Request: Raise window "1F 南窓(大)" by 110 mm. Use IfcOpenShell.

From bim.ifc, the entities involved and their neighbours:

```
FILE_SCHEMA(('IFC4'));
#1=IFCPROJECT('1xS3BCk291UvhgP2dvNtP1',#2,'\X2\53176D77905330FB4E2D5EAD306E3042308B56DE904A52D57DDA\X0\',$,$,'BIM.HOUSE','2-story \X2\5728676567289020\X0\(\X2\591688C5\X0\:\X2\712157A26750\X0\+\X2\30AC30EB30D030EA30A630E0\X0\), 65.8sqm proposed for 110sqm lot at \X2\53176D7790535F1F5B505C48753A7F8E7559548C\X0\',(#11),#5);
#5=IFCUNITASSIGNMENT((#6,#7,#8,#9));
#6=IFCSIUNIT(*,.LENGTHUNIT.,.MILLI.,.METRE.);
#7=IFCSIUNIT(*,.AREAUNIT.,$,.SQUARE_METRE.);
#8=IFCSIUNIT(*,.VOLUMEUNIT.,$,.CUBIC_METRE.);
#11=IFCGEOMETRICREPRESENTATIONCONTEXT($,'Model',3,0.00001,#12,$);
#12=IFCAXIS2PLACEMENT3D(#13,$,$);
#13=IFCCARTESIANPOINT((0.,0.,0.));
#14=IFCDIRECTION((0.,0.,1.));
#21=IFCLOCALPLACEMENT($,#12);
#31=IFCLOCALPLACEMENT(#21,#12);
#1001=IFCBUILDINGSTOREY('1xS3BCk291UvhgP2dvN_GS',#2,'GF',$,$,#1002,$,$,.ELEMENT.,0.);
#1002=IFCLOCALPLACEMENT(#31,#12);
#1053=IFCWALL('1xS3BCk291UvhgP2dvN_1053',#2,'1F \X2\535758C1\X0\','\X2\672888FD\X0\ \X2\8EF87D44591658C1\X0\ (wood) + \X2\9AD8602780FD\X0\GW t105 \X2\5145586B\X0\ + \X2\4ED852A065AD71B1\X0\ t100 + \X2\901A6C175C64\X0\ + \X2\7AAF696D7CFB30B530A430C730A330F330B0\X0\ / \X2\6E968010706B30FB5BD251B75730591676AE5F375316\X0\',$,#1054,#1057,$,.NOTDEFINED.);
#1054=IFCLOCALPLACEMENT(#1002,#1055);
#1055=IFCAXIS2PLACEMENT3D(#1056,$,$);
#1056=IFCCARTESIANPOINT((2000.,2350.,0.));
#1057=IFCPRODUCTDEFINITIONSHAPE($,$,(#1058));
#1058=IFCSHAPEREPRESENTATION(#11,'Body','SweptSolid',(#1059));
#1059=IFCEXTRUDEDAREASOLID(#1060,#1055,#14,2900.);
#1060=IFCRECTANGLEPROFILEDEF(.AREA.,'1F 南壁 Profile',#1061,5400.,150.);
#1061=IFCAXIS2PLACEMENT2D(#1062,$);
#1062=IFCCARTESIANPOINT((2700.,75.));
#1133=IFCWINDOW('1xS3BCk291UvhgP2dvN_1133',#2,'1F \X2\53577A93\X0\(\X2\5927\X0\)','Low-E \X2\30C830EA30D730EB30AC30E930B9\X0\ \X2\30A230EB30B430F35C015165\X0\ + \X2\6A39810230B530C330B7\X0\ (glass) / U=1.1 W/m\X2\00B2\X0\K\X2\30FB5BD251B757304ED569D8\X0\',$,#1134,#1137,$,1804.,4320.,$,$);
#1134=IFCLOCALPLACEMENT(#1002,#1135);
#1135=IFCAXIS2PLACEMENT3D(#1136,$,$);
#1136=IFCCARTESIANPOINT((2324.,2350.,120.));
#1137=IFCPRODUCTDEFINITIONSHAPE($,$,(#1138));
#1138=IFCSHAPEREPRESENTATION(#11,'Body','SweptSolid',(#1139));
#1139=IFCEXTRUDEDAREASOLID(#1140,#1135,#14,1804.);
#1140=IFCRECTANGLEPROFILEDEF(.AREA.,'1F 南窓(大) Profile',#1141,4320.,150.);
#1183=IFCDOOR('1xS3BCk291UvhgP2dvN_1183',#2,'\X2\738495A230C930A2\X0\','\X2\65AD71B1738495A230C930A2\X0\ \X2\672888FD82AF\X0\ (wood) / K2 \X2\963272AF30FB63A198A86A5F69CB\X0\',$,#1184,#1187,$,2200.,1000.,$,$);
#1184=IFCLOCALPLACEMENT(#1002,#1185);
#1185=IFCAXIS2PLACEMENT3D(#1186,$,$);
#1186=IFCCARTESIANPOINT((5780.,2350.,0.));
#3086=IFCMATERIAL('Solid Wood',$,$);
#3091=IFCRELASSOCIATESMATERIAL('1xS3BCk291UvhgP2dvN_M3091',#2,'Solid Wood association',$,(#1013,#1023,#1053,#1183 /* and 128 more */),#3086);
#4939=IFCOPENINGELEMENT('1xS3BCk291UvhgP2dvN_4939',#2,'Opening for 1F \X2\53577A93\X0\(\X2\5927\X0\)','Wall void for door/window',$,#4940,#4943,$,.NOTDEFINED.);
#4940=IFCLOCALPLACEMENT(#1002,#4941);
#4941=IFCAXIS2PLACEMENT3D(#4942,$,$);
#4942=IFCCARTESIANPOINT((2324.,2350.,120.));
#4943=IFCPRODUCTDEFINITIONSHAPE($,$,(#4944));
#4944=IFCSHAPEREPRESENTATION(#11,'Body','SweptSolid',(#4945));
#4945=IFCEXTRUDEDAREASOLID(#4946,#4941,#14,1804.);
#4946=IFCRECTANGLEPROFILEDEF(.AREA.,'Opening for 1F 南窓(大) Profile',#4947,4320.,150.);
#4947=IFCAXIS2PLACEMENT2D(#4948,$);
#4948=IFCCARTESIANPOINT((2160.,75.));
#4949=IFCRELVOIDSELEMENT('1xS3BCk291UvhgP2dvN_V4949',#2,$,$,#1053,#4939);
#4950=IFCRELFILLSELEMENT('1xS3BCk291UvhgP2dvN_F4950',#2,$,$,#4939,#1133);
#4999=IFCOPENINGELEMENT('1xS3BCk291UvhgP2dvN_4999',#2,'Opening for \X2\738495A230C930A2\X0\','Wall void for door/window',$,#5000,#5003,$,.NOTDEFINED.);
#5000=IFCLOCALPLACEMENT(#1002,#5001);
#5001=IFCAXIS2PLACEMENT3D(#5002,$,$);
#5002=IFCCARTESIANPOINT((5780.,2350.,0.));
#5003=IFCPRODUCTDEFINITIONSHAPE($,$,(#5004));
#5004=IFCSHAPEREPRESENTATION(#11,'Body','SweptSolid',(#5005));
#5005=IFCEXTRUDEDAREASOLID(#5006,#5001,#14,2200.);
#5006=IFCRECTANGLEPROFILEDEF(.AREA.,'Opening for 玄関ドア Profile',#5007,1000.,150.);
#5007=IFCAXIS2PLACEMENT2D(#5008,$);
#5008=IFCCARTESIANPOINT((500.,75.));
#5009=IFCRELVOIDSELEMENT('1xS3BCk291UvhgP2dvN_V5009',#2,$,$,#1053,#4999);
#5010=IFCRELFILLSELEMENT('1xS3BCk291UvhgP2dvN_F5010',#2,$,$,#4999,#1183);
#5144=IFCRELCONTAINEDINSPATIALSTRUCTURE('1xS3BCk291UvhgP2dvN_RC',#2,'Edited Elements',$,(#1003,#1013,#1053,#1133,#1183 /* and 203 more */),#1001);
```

```python
import numpy as np
import ifcopenshell
import ifcopenshell.api.geometry
import ifcopenshell.util.placement
import ifcopenshell.util.unit

model = ifcopenshell.open("bim.ifc")
unit_scale = ifcopenshell.util.unit.calculate_unit_scale(model)

window = model.by_id(1133)
opening = window.FillsVoids[0].RelatingOpeningElement
dz = 0.11 / unit_scale

shift = np.array([0.0, 0.0, dz])
# The window is not placed relative to its opening, so move both.
for product in (opening, window):
    matrix = ifcopenshell.util.placement.get_local_placement(product.ObjectPlacement)
    matrix[:3, 3] += shift
    ifcopenshell.api.geometry.edit_object_placement(model, product=product, matrix=matrix, is_si=False)

print(f"moved by {dz * unit_scale:+.3f} m")

model.write("bim_updated.ifc")
```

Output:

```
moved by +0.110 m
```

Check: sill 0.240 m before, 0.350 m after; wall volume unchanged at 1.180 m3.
